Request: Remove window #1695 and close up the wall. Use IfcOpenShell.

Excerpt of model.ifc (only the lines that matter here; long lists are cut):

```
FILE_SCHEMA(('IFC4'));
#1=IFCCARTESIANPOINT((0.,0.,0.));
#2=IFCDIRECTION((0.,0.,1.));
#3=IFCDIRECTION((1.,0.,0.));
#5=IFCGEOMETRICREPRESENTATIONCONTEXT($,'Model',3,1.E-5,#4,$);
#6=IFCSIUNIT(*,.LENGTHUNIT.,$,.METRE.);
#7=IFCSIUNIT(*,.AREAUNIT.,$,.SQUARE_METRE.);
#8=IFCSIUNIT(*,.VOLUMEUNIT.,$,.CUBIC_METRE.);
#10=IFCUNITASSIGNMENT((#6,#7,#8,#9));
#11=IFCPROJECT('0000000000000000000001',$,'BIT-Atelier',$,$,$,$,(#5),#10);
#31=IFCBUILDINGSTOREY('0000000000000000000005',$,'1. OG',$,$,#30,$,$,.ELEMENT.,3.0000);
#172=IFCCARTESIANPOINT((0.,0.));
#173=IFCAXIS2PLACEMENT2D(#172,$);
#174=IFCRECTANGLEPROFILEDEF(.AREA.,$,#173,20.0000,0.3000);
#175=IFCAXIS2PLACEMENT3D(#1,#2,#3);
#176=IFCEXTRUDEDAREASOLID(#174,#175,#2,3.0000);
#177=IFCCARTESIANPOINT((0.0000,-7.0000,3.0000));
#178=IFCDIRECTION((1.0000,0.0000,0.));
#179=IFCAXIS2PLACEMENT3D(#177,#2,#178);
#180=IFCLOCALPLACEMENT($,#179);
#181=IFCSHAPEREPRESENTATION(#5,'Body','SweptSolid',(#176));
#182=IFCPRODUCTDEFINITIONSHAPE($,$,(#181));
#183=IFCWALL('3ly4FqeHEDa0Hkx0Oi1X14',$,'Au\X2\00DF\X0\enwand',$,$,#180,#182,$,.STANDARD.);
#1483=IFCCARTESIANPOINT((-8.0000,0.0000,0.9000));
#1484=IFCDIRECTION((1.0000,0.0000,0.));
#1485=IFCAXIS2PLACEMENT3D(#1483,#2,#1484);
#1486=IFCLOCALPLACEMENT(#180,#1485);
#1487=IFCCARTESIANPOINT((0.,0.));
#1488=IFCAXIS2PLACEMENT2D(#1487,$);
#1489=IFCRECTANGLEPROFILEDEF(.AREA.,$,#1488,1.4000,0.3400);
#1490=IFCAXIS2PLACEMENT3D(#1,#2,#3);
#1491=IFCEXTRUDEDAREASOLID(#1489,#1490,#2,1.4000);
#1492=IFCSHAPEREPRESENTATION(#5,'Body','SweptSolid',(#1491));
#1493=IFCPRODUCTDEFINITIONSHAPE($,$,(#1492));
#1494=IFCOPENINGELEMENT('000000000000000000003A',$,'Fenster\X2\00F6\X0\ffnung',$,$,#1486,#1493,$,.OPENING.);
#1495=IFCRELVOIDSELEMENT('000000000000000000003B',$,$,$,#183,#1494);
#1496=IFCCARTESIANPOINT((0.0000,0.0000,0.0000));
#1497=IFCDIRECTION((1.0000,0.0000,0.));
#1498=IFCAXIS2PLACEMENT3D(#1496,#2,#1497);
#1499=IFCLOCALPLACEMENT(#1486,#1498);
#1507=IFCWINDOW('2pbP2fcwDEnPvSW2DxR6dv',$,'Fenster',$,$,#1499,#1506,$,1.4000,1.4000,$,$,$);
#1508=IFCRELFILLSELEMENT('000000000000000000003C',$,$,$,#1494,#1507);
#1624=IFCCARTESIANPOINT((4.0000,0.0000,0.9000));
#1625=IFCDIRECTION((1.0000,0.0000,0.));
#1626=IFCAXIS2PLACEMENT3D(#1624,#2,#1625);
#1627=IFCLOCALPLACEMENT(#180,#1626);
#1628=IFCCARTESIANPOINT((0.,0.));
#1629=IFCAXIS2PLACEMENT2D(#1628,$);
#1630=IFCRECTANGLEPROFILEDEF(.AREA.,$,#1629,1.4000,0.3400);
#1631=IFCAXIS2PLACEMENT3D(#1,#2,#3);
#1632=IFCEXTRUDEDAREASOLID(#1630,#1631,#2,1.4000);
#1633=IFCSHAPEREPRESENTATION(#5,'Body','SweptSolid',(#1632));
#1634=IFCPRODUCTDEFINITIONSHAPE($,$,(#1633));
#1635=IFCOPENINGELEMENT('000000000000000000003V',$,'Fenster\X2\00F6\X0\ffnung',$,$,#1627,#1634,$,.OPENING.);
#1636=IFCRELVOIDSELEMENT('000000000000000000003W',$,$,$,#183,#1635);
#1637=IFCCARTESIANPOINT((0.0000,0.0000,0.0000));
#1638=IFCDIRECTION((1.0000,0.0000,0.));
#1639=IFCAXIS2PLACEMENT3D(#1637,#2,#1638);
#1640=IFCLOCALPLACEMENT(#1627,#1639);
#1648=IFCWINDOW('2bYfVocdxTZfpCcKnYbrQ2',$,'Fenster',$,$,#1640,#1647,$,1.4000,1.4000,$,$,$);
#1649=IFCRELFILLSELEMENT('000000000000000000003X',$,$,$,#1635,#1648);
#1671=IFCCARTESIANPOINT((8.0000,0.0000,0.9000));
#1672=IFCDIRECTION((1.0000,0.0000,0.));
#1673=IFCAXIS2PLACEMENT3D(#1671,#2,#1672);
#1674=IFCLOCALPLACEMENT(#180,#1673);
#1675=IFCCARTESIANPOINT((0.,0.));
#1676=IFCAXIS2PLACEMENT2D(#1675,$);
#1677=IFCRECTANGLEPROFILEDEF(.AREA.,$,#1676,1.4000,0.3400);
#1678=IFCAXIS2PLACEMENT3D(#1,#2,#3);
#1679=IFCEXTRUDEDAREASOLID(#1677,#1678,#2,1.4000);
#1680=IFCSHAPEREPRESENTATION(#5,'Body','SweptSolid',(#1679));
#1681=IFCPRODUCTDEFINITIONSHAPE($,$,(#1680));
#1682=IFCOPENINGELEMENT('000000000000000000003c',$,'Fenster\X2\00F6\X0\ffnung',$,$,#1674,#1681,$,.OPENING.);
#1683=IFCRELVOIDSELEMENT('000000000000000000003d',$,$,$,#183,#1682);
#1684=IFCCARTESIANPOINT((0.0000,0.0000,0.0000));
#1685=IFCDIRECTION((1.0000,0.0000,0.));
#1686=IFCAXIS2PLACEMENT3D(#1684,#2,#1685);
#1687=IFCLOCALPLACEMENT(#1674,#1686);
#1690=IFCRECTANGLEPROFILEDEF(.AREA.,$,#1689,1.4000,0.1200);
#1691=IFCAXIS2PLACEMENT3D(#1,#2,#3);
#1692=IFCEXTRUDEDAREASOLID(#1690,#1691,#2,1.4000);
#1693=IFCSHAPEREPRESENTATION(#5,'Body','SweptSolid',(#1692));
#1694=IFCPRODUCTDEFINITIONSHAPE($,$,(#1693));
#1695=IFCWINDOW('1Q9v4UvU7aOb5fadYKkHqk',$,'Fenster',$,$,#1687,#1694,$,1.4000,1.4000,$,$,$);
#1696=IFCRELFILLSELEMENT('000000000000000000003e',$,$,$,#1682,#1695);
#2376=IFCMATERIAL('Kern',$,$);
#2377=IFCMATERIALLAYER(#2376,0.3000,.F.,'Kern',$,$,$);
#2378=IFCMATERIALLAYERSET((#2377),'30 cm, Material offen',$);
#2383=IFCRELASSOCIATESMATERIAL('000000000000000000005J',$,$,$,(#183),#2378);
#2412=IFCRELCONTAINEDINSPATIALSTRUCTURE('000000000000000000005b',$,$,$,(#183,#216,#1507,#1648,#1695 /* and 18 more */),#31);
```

```python
import ifcopenshell
import ifcopenshell.api.feature
import ifcopenshell.api.root
import ifcopenshell.geom
import ifcopenshell.util.shape

model = ifcopenshell.open("model.ifc")
settings = ifcopenshell.geom.settings()


def volume(element):
    """Net volume in cubic metres, openings subtracted."""
    shape = ifcopenshell.geom.create_shape(settings, element)
    return ifcopenshell.util.shape.get_volume(shape.geometry)


window = model.by_guid("1Q9v4UvU7aOb5fadYKkHqk")
opening = window.FillsVoids[0].RelatingOpeningElement
wall = opening.VoidsElements[0].RelatingBuildingElement
before = volume(wall)

ifcopenshell.api.root.remove_product(model, product=window)
ifcopenshell.api.feature.remove_feature(model, feature=opening)

after = volume(wall)

print(f"wall volume {before:.3f} -> {after:.3f} m3")

model.write("model_edited.ifc")
```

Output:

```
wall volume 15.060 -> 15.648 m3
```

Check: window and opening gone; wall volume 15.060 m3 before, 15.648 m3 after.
